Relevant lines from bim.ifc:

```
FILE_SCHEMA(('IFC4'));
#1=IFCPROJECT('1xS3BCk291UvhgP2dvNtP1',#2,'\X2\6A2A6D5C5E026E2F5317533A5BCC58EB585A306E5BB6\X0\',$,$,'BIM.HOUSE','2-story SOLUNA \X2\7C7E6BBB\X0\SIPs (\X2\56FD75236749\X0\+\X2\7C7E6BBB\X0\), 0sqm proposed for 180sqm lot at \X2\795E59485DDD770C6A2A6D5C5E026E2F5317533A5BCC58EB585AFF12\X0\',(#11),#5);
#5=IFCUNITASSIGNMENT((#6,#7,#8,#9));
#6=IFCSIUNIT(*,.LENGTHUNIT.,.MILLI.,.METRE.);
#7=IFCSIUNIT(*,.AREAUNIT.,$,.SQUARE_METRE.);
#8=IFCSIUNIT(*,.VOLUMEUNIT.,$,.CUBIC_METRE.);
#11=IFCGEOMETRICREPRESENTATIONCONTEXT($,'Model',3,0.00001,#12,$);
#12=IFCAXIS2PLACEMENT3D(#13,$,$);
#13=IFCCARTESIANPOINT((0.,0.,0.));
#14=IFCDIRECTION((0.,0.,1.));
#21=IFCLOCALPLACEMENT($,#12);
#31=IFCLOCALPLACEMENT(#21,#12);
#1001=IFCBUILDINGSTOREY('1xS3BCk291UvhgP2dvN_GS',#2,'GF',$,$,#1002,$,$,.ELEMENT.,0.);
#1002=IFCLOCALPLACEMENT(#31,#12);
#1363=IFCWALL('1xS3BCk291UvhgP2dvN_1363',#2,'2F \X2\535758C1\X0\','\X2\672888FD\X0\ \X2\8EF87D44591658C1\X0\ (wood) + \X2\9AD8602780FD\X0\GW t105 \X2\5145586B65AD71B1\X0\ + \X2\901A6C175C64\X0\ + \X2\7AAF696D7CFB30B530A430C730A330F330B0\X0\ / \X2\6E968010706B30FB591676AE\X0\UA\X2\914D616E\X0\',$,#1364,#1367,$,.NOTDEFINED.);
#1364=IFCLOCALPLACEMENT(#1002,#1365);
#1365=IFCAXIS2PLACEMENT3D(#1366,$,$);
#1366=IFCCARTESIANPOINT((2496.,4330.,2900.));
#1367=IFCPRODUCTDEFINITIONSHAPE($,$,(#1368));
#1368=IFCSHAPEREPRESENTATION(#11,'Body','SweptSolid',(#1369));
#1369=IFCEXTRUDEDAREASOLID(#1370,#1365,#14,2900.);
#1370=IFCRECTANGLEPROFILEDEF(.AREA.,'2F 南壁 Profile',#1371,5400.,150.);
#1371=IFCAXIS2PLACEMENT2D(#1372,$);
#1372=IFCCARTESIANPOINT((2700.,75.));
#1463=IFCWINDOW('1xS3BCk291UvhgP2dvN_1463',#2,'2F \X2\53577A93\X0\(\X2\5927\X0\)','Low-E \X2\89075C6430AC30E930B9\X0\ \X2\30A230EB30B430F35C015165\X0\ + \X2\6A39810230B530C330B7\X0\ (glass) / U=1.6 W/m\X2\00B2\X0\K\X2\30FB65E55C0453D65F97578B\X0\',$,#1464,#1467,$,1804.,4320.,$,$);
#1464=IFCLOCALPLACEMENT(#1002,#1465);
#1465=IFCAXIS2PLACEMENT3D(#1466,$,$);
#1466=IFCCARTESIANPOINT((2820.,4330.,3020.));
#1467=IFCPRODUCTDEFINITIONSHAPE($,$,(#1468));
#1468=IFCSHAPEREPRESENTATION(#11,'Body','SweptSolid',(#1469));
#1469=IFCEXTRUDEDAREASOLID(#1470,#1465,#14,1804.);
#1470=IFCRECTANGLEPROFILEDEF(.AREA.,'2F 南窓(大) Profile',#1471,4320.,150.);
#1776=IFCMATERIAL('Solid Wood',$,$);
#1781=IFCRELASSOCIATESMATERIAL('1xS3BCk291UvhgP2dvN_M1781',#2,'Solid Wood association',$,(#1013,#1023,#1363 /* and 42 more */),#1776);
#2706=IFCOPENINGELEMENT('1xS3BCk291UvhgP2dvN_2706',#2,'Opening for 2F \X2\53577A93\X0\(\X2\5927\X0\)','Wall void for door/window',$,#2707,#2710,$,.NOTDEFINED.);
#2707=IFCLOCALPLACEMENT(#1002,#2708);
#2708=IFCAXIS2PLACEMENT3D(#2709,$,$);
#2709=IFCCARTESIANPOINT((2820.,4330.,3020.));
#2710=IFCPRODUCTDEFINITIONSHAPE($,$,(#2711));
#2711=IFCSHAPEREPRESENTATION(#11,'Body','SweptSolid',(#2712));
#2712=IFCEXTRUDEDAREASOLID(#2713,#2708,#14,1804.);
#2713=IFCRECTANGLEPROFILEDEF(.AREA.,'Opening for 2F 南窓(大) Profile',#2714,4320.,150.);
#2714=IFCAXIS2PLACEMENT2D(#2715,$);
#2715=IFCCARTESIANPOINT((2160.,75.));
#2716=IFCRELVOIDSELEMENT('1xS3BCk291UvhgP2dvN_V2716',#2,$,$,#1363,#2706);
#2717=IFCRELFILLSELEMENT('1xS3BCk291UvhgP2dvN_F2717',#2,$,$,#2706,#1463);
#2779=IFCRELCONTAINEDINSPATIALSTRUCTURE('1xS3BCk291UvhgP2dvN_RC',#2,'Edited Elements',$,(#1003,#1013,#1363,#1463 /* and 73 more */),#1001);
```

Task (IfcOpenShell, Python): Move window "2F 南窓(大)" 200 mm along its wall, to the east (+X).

```python
import ifcopenshell
import ifcopenshell.api.geometry
import ifcopenshell.util.placement
import ifcopenshell.util.unit

model = ifcopenshell.open("bim.ifc")
unit_scale = ifcopenshell.util.unit.calculate_unit_scale(model)

window = model.by_guid("1xS3BCk291UvhgP2dvN_1463")
opening = window.FillsVoids[0].RelatingOpeningElement
wall = opening.VoidsElements[0].RelatingBuildingElement

wall_matrix = ifcopenshell.util.placement.get_local_placement(wall.ObjectPlacement)
shift = wall_matrix[:3, 0] * 0.2 / unit_scale
before = ifcopenshell.util.placement.get_local_placement(window.ObjectPlacement)[:3, 3].copy()

# The window is not placed relative to its opening, so move both.
for product in (opening, window):
    matrix = ifcopenshell.util.placement.get_local_placement(product.ObjectPlacement)
    matrix[:3, 3] += shift
    ifcopenshell.api.geometry.edit_object_placement(model, product=product, matrix=matrix, is_si=False)

after = ifcopenshell.util.placement.get_local_placement(window.ObjectPlacement)[:3, 3]
print("window moved by", (after - before).round(3) + 0.0)

model.write("bim_rev.ifc")
```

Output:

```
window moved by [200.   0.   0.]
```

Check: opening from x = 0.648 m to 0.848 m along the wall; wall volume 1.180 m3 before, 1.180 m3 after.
